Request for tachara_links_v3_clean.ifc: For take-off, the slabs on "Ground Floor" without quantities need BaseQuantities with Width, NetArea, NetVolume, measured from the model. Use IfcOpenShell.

First a look at what the model holds.

```python
import ifcopenshell
import ifcopenshell.util.element
import ifcopenshell.util.unit

model = ifcopenshell.open("tachara_links_v3_clean.ifc")
print(model.schema)
for unit_type in ("LENGTHUNIT", "AREAUNIT", "VOLUMEUNIT"):
    print(unit_type, ifcopenshell.util.unit.calculate_unit_scale(model, unit_type))
storey = next(s for s in model.by_type("IfcBuildingStorey") if s.Name == "Ground Floor")
slabs = [e for e in ifcopenshell.util.element.get_decomposition(storey) if e.is_a("IfcSlab")]
for e in sorted(slabs, key=lambda e: e.id()):
    print(e.id(), e.is_a(), e.Name, list(ifcopenshell.util.element.get_psets(e, qtos_only=True)), sep=" | ")
```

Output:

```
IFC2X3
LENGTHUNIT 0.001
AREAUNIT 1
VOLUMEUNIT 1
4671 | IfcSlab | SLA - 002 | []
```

```python
import ifcopenshell
import ifcopenshell.api.pset
import ifcopenshell.geom
import ifcopenshell.util.element
import ifcopenshell.util.shape
import ifcopenshell.util.unit

model = ifcopenshell.open("tachara_links_v3_clean.ifc")
unit_scale = ifcopenshell.util.unit.calculate_unit_scale(model)
area_scale = ifcopenshell.util.unit.calculate_unit_scale(model, "AREAUNIT")
volume_scale = ifcopenshell.util.unit.calculate_unit_scale(model, "VOLUMEUNIT")
settings = ifcopenshell.geom.settings()

storey = next(s for s in model.by_type("IfcBuildingStorey") if s.Name == "Ground Floor")
slabs = [e for e in ifcopenshell.util.element.get_decomposition(storey) if e.is_a("IfcSlab")]

for e in sorted(slabs, key=lambda e: e.id()):
    if ifcopenshell.util.element.get_psets(e, qtos_only=True, should_inherit=False):
        continue
    # Geometry comes back in metres, in the element's own axes.
    shape = ifcopenshell.geom.create_shape(settings, e)
    values = {
        "Width": ifcopenshell.util.shape.get_z(shape.geometry) / unit_scale,
        "NetArea": ifcopenshell.util.shape.get_footprint_area(shape.geometry) / area_scale,
        "NetVolume": ifcopenshell.util.shape.get_volume(shape.geometry) / volume_scale,
    }
    qto = ifcopenshell.api.pset.add_qto(model, product=e, name="BaseQuantities")
    ifcopenshell.api.pset.edit_qto(model, qto=qto, properties=values)
    print(e.id(), {k: round(v, 3) for k, v in values.items()})

model.write("tachara_links_v3_clean_rev.ifc")
```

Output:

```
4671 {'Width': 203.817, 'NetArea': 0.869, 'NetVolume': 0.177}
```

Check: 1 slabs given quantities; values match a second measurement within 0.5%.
